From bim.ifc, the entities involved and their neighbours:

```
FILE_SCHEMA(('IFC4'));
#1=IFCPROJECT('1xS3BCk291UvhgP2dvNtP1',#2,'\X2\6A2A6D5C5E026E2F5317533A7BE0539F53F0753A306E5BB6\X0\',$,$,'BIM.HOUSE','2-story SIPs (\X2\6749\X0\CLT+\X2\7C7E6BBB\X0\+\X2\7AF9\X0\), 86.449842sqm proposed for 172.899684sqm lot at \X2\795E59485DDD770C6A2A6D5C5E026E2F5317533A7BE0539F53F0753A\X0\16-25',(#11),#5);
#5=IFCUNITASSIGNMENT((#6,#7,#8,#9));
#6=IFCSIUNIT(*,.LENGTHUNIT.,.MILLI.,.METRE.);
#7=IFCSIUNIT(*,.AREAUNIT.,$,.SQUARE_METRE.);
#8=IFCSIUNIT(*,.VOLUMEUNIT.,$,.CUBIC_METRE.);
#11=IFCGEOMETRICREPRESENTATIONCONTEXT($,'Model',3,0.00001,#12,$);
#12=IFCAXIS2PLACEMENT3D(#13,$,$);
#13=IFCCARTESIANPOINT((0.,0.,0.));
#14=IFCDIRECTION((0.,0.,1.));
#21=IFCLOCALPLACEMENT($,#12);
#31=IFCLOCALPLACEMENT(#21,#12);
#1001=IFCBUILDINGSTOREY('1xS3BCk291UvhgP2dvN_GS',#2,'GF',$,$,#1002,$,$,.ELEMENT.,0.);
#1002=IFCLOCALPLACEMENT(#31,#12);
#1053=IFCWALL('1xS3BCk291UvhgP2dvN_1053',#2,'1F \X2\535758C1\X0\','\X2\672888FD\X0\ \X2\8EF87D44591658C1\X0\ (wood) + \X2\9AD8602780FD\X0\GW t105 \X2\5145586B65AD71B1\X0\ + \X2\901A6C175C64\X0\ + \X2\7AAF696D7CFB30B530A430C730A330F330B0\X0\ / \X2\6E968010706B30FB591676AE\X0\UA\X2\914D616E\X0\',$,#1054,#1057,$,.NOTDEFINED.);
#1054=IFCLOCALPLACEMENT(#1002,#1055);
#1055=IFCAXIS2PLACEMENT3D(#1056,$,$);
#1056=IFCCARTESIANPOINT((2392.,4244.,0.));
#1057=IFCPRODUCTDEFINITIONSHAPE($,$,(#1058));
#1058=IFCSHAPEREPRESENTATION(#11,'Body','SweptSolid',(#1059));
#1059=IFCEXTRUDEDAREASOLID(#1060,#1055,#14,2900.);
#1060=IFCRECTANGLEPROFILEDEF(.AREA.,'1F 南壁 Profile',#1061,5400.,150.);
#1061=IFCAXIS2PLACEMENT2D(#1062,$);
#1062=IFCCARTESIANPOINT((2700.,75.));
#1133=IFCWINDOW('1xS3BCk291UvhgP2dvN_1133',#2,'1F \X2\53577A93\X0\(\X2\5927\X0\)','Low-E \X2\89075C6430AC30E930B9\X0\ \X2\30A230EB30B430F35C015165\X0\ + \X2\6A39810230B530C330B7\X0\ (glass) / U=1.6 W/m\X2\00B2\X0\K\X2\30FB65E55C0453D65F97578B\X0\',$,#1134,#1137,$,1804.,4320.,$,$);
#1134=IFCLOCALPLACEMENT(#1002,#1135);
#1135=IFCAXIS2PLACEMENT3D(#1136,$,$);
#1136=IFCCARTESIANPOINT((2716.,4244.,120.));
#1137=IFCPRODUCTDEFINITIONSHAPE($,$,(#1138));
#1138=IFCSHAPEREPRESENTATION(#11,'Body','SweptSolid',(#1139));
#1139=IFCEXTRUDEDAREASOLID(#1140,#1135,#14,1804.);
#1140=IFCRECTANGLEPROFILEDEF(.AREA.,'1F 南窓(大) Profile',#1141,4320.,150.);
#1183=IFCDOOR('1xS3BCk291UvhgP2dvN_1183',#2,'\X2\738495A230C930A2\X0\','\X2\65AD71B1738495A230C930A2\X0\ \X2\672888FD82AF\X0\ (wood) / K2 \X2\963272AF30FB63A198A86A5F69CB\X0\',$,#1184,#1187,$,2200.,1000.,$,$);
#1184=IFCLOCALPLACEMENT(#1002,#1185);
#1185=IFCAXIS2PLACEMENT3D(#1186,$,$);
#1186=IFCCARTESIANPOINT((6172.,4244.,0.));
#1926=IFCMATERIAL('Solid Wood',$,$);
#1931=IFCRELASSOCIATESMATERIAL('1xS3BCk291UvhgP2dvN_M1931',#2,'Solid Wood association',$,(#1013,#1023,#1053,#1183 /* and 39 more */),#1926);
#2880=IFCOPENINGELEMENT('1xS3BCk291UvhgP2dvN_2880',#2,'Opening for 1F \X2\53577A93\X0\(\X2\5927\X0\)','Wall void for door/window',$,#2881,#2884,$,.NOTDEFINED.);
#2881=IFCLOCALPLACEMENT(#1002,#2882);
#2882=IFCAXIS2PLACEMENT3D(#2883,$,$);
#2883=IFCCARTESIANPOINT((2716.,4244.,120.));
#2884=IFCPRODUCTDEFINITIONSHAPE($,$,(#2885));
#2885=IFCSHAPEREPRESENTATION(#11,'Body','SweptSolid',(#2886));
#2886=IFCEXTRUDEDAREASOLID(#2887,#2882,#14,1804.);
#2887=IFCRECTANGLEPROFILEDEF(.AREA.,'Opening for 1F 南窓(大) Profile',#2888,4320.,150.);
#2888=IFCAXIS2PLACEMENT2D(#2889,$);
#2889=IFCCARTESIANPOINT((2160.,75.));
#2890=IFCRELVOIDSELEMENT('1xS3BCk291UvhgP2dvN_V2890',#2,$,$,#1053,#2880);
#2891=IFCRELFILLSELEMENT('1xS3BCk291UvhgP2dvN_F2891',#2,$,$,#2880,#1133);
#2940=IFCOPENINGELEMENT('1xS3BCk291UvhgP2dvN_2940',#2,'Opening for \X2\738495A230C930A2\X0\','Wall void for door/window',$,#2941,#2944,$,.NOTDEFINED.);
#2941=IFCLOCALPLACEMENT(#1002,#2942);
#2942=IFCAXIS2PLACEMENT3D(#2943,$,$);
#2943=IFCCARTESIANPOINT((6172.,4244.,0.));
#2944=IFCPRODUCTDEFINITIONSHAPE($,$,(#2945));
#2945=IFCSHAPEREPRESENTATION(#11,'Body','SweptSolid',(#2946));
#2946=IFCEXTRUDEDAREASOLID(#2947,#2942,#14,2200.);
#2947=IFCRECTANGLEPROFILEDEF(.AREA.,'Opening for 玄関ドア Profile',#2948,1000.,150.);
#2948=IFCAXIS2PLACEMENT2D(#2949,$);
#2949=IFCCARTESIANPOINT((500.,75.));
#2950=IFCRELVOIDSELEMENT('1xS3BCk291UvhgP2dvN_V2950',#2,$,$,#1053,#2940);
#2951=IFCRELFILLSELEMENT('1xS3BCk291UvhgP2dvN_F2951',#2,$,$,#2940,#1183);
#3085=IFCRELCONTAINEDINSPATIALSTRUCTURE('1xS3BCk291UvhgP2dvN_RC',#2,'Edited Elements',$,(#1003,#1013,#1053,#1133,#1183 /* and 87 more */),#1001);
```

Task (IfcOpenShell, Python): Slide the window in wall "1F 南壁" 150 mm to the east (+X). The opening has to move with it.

```python
import ifcopenshell
import ifcopenshell.api.geometry
import ifcopenshell.util.placement

model = ifcopenshell.open("bim.ifc")

window = model.by_guid("1xS3BCk291UvhgP2dvN_1133")
opening = window.FillsVoids[0].RelatingOpeningElement
wall = opening.VoidsElements[0].RelatingBuildingElement

wall_matrix = ifcopenshell.util.placement.get_local_placement(wall.ObjectPlacement)
shift = wall_matrix[:3, 0] * 150.0
before = ifcopenshell.util.placement.get_local_placement(window.ObjectPlacement)[:3, 3].copy()

# The window is not placed relative to its opening, so move both.
for product in (opening, window):
    matrix = ifcopenshell.util.placement.get_local_placement(product.ObjectPlacement)
    matrix[:3, 3] += shift
    ifcopenshell.api.geometry.edit_object_placement(model, product=product, matrix=matrix, is_si=False)

after = ifcopenshell.util.placement.get_local_placement(window.ObjectPlacement)[:3, 3]
print("window moved by", (after - before).round(3) + 0.0)

model.write("bim_rev.ifc")
```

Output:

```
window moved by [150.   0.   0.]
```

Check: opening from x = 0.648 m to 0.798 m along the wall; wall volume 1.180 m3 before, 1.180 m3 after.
